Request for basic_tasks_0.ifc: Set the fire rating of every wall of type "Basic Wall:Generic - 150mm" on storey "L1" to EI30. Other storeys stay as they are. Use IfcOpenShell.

First a look at what the model holds.

```python
import ifcopenshell
import ifcopenshell.util.element

model = ifcopenshell.open("basic_tasks_0.ifc")
print(model.schema)
storey = next(s for s in model.by_type("IfcBuildingStorey") if s.Name == "L1")
walls = [e for e in ifcopenshell.util.element.get_decomposition(storey) if e.is_a("IfcWall")]
seen = {}
for e in walls:
    element_type = ifcopenshell.util.element.get_type(e)
    key = (element_type.Name if element_type != e and element_type else None, ifcopenshell.util.element.get_pset(e, "Pset_WallCommon", "FireRating"))
    seen[key] = seen.get(key, 0) + 1
for (name, value), count in sorted(seen.items(), key=str):
    print(count, "x", name, "|", value)
```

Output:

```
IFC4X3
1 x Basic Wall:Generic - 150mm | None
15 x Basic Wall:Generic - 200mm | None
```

```python
import ifcopenshell
import ifcopenshell.api.pset
import ifcopenshell.util.element

model = ifcopenshell.open("basic_tasks_0.ifc")

storey = next(s for s in model.by_type("IfcBuildingStorey") if s.Name == "L1")
walls = [e for e in ifcopenshell.util.element.get_decomposition(storey) if e.is_a("IfcWall")]

count = 0
for e in walls:
    element_type = ifcopenshell.util.element.get_type(e)
    if element_type in (None, e) or element_type.Name != "Basic Wall:Generic - 150mm":
        continue
    # add_pset returns the element's existing set when there is one.
    pset = ifcopenshell.api.pset.add_pset(model, product=e, name="Pset_WallCommon")
    ifcopenshell.api.pset.edit_pset(model, pset=pset, properties={"FireRating": "EI30"})
    count += 1

print(count, "walls updated")

model.write("basic_tasks_0-out.ifc")
```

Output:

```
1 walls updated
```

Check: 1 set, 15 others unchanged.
